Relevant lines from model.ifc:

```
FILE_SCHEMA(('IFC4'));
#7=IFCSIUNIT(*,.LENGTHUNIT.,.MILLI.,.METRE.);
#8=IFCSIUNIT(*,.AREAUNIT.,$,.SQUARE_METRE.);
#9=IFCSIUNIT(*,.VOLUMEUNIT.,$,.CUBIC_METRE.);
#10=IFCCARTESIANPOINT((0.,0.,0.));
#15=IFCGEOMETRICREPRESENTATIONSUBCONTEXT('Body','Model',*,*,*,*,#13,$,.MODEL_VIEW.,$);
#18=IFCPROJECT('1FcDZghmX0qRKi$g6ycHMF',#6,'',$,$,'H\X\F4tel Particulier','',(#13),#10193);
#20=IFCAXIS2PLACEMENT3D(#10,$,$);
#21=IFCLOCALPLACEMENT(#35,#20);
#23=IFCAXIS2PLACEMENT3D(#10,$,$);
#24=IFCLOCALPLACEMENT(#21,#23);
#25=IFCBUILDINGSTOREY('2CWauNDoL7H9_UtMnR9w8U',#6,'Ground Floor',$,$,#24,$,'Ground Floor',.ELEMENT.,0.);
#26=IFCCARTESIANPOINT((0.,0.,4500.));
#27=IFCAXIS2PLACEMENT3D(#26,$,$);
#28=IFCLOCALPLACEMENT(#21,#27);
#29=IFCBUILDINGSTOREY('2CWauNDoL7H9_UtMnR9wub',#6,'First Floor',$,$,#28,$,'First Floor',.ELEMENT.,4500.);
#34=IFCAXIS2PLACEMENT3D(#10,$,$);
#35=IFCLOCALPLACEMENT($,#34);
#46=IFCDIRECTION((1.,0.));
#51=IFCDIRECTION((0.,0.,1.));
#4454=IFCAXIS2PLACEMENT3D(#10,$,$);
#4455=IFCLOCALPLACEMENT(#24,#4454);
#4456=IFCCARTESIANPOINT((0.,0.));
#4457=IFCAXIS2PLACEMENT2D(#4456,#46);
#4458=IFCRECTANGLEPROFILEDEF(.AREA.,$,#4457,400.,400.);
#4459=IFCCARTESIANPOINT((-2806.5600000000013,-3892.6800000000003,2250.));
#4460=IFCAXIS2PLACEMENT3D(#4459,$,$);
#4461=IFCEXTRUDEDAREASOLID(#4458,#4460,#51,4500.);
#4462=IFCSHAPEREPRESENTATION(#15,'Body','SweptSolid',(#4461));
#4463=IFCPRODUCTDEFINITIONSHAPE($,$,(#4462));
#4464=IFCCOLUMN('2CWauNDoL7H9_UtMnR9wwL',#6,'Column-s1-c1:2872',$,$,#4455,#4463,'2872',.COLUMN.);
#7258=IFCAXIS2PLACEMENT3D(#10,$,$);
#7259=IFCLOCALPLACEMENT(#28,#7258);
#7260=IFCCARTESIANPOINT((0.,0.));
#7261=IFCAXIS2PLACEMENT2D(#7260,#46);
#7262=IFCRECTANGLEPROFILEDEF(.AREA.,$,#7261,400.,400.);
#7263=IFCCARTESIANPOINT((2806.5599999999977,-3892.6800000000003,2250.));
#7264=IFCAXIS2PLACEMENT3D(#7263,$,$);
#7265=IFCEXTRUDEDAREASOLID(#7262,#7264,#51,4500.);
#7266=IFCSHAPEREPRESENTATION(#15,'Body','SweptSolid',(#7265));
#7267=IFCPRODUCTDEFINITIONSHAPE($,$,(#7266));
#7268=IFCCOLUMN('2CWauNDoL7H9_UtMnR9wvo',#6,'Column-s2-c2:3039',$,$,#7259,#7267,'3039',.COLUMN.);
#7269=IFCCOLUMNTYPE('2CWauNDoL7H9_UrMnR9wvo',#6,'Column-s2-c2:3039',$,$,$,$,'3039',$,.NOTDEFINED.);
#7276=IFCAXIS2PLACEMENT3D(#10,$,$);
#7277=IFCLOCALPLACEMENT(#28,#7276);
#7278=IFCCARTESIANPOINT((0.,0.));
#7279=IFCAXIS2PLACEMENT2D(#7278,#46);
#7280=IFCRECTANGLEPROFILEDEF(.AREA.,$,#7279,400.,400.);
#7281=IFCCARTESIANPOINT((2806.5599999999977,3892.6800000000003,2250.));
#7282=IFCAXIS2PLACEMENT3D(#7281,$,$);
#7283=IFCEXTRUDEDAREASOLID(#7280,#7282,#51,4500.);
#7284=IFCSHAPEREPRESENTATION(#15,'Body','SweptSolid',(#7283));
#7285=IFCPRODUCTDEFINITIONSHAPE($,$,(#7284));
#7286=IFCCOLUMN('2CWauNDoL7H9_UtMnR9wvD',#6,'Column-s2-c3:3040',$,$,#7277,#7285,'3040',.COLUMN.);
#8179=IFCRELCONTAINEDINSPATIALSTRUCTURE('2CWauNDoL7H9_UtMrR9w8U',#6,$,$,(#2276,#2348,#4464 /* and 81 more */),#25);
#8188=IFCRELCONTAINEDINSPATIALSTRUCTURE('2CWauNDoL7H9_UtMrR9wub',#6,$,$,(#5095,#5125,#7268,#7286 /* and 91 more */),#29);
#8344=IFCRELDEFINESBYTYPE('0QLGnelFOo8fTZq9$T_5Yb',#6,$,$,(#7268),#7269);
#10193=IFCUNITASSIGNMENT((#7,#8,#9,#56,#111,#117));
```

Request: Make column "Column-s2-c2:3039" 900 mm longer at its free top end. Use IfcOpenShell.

```python
import ifcopenshell
import ifcopenshell.util.representation

model = ifcopenshell.open("model.ifc")

member = model.by_id(7268)
change = 900.0

# The extrusion runs towards the end named, so only its depth changes.
body = ifcopenshell.util.representation.get_representation(member, "Model", "Body")
solid = body.Items[0]
old_length = solid.Depth
solid.Depth += change

print(f"length {old_length:g} -> {solid.Depth:g}")

model.write("model_updated.ifc")
```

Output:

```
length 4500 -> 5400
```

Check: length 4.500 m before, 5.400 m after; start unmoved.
